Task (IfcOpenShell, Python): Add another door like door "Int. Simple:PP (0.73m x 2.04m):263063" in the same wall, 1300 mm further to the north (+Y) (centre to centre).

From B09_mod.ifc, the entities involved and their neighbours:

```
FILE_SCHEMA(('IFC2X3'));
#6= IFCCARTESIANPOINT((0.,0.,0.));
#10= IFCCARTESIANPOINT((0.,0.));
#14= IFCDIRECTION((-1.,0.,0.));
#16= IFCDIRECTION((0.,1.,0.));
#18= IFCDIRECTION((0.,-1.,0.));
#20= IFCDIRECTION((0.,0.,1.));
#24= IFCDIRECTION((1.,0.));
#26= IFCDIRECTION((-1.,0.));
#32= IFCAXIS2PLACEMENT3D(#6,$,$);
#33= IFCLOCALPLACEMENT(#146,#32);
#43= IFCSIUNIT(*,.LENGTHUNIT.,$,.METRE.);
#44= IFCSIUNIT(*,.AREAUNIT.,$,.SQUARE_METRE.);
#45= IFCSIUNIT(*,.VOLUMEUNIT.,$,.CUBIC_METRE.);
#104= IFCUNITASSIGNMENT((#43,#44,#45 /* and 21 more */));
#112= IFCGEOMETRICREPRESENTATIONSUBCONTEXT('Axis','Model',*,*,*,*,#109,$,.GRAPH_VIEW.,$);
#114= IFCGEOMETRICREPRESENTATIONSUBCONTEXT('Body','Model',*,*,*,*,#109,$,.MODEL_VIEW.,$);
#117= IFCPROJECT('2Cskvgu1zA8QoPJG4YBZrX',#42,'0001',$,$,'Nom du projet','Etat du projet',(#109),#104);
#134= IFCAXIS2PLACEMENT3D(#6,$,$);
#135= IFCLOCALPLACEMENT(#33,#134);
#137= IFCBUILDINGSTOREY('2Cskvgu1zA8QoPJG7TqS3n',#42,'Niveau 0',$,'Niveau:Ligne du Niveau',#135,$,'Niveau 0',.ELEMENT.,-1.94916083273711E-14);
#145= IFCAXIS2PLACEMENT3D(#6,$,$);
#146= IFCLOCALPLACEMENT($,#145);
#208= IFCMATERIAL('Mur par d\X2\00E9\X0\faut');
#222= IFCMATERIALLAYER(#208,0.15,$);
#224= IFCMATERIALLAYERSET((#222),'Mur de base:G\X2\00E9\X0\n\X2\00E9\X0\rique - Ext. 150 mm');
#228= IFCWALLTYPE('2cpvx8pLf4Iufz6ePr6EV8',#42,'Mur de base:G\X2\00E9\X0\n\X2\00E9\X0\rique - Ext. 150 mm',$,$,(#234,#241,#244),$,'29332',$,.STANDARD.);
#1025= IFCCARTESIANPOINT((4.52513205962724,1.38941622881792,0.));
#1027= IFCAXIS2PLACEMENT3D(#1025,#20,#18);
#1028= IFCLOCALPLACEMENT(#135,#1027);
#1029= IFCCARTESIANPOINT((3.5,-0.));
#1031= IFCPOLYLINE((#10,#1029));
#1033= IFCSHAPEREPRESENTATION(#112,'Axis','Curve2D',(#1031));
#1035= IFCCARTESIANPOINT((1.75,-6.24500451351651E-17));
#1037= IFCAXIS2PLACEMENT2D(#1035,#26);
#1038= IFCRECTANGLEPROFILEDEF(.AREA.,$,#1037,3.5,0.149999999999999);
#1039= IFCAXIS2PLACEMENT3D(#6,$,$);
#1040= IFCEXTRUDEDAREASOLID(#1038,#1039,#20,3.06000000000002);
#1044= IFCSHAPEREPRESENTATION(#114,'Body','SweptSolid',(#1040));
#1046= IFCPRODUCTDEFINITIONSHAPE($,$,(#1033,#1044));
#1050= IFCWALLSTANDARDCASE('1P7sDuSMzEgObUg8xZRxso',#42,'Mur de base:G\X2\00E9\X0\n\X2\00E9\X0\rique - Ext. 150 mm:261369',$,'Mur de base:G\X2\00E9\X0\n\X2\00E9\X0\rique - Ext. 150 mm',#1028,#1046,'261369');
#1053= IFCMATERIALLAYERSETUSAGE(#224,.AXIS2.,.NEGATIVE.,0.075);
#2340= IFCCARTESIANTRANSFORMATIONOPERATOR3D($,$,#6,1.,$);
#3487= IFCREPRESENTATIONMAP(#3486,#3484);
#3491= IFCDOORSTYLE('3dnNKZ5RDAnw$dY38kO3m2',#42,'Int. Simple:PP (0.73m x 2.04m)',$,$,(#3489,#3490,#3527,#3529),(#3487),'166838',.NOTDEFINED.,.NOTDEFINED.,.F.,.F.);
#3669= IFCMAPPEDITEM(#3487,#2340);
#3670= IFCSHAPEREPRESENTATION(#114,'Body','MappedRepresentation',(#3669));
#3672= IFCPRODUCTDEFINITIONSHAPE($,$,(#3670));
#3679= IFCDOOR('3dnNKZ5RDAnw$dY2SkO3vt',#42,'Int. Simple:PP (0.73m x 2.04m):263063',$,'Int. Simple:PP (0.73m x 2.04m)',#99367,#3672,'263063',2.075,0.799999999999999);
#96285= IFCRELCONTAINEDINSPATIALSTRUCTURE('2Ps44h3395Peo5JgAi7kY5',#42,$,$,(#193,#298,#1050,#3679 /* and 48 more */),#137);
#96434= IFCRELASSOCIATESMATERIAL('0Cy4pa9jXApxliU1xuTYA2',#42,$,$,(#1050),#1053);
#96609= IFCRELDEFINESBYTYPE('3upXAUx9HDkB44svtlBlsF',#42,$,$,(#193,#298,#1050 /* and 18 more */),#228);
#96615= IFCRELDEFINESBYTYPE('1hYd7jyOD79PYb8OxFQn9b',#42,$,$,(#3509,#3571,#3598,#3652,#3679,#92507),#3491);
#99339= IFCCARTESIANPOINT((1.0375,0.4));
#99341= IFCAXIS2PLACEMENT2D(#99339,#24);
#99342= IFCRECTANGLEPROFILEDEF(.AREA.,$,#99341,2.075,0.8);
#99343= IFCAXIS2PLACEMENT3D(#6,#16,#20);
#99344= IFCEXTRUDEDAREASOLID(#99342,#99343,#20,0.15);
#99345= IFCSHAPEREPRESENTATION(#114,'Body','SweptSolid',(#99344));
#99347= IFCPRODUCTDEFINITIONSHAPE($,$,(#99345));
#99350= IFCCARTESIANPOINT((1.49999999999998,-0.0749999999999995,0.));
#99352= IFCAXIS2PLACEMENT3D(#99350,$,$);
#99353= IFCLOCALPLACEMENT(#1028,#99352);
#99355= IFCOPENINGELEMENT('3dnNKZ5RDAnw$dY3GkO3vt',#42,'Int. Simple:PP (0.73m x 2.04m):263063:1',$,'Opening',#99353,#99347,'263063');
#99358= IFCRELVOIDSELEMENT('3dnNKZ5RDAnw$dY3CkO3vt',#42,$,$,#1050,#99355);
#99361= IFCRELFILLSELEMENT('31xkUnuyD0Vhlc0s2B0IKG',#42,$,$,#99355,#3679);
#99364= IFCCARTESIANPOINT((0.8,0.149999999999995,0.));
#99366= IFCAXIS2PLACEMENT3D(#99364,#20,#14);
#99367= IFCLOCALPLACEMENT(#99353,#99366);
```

```python
import ifcopenshell
import ifcopenshell.api.feature
import ifcopenshell.api.geometry
import ifcopenshell.api.root
import ifcopenshell.geom
import ifcopenshell.util.element
import ifcopenshell.util.placement
import ifcopenshell.util.shape
import ifcopenshell.util.unit

model = ifcopenshell.open("B09_mod.ifc")
unit_scale = ifcopenshell.util.unit.calculate_unit_scale(model)
settings = ifcopenshell.geom.settings()


def volume(element):
    """Net volume in cubic metres, openings subtracted."""
    shape = ifcopenshell.geom.create_shape(settings, element)
    return ifcopenshell.util.shape.get_volume(shape.geometry)


def reuse_history(source, copy):
    """copy_class also copies each property set's owner history, people and application; keep the originals."""
    for rel in copy.IsDefinedBy:
        if rel.is_a("IfcRelDefinesByProperties") and (history := rel.RelatingPropertyDefinition.OwnerHistory):
            rel.RelatingPropertyDefinition.OwnerHistory = source.OwnerHistory
            ifcopenshell.util.element.remove_deep2(model, history)


door = model.by_id(3679)
opening = door.FillsVoids[0].RelatingOpeningElement
wall = opening.VoidsElements[0].RelatingBuildingElement
before = volume(wall)
shift = ifcopenshell.util.placement.get_local_placement(wall.ObjectPlacement)[:3, 0] * -1.3 / unit_scale

# copy_class copies the void relationship, type, container and properties, but no geometry.
new_opening = ifcopenshell.api.root.copy_class(model, product=opening)
new_opening.Representation = ifcopenshell.util.element.copy_deep(
    model, opening.Representation, exclude=["IfcGeometricRepresentationContext", "IfcRepresentationMap"]
)
new_opening.Name = "Int. Simple:PP (0.73m x 2.04m)"
new_opening.Tag = None
new_door = ifcopenshell.api.root.copy_class(model, product=door)
new_door.Representation = ifcopenshell.util.element.copy_deep(
    model, door.Representation, exclude=["IfcGeometricRepresentationContext", "IfcRepresentationMap"]
)
new_door.Name = "Int. Simple:PP (0.73m x 2.04m)"
new_door.Tag = None
reuse_history(door, new_door)
fills = ifcopenshell.api.feature.add_filling(model, opening=new_opening, element=new_door)
fills.OwnerHistory = new_door.OwnerHistory  # required in IFC2X3

for old, new in ((opening, new_opening), (door, new_door)):
    matrix = ifcopenshell.util.placement.get_local_placement(old.ObjectPlacement)
    matrix[:3, 3] += shift
    ifcopenshell.api.geometry.edit_object_placement(model, product=new, matrix=matrix, is_si=False)

after = volume(wall)

print(f"wall volume {before:.3f} -> {after:.3f} m3")

model.write("B09_mod-out.ifc")
```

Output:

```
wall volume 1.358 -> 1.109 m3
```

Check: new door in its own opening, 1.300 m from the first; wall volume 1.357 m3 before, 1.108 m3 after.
